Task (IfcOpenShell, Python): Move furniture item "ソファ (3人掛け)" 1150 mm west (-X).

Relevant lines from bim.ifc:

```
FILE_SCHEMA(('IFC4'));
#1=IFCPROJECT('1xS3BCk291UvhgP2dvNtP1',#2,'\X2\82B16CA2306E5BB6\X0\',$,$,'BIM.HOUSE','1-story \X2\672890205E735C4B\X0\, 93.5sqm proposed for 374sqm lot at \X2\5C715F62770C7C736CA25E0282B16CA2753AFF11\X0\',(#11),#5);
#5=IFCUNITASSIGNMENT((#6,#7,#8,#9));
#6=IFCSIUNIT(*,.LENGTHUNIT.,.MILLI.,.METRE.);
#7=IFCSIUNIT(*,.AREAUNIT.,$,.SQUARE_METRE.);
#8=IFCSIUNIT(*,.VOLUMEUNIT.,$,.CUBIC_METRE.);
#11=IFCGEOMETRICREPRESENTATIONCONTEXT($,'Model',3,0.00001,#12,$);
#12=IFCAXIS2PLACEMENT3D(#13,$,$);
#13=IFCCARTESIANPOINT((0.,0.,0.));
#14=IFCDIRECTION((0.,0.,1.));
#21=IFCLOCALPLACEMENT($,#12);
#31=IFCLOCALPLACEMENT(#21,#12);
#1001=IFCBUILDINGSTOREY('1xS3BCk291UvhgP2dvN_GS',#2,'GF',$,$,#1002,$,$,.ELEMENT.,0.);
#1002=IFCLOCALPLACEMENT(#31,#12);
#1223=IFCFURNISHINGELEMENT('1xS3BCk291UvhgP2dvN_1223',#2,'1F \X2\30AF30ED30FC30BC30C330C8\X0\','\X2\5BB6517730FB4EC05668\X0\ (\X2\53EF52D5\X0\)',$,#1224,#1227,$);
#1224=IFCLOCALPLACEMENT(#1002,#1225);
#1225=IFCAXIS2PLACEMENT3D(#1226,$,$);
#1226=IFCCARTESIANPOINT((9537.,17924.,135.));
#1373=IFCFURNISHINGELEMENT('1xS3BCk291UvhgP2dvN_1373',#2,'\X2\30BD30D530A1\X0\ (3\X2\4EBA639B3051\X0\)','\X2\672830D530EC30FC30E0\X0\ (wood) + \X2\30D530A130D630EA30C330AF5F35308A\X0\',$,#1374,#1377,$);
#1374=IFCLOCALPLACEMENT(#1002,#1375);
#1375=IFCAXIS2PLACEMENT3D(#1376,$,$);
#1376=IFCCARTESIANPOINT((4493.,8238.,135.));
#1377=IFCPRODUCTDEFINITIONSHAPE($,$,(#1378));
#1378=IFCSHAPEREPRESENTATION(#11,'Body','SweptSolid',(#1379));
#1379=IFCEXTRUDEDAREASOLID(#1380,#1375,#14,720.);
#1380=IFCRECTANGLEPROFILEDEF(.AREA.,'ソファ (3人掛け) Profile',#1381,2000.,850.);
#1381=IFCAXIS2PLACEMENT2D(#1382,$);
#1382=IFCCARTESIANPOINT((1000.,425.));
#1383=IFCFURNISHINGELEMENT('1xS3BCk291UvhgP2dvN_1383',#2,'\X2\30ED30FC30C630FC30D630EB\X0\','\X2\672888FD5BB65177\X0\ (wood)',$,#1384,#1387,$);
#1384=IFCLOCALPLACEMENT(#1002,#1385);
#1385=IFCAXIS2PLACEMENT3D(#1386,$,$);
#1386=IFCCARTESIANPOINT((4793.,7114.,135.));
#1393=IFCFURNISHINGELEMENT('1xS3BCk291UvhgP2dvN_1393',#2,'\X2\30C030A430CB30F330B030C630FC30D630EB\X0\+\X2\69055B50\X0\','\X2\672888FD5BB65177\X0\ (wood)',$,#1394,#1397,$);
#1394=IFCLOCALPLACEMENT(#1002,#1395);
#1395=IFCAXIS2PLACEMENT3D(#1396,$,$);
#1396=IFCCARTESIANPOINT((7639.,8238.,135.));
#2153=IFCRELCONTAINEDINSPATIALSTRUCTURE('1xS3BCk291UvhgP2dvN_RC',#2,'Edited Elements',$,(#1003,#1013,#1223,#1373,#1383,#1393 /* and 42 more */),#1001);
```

```python
import ifcopenshell
import ifcopenshell.api.geometry
import ifcopenshell.util.placement

model = ifcopenshell.open("bim.ifc")

item = model.by_guid("1xS3BCk291UvhgP2dvN_1373")
matrix = ifcopenshell.util.placement.get_local_placement(item.ObjectPlacement)
matrix[0, 3] -= 1150.0
ifcopenshell.api.geometry.edit_object_placement(model, product=item, matrix=matrix, is_si=False)

print(ifcopenshell.util.placement.get_local_placement(item.ObjectPlacement).round(3) + 0.0)

model.write("bim_updated.ifc")
```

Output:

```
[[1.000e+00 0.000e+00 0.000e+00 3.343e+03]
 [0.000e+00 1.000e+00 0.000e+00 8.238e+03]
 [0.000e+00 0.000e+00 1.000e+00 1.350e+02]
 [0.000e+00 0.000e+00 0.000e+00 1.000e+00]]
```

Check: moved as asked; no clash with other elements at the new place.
